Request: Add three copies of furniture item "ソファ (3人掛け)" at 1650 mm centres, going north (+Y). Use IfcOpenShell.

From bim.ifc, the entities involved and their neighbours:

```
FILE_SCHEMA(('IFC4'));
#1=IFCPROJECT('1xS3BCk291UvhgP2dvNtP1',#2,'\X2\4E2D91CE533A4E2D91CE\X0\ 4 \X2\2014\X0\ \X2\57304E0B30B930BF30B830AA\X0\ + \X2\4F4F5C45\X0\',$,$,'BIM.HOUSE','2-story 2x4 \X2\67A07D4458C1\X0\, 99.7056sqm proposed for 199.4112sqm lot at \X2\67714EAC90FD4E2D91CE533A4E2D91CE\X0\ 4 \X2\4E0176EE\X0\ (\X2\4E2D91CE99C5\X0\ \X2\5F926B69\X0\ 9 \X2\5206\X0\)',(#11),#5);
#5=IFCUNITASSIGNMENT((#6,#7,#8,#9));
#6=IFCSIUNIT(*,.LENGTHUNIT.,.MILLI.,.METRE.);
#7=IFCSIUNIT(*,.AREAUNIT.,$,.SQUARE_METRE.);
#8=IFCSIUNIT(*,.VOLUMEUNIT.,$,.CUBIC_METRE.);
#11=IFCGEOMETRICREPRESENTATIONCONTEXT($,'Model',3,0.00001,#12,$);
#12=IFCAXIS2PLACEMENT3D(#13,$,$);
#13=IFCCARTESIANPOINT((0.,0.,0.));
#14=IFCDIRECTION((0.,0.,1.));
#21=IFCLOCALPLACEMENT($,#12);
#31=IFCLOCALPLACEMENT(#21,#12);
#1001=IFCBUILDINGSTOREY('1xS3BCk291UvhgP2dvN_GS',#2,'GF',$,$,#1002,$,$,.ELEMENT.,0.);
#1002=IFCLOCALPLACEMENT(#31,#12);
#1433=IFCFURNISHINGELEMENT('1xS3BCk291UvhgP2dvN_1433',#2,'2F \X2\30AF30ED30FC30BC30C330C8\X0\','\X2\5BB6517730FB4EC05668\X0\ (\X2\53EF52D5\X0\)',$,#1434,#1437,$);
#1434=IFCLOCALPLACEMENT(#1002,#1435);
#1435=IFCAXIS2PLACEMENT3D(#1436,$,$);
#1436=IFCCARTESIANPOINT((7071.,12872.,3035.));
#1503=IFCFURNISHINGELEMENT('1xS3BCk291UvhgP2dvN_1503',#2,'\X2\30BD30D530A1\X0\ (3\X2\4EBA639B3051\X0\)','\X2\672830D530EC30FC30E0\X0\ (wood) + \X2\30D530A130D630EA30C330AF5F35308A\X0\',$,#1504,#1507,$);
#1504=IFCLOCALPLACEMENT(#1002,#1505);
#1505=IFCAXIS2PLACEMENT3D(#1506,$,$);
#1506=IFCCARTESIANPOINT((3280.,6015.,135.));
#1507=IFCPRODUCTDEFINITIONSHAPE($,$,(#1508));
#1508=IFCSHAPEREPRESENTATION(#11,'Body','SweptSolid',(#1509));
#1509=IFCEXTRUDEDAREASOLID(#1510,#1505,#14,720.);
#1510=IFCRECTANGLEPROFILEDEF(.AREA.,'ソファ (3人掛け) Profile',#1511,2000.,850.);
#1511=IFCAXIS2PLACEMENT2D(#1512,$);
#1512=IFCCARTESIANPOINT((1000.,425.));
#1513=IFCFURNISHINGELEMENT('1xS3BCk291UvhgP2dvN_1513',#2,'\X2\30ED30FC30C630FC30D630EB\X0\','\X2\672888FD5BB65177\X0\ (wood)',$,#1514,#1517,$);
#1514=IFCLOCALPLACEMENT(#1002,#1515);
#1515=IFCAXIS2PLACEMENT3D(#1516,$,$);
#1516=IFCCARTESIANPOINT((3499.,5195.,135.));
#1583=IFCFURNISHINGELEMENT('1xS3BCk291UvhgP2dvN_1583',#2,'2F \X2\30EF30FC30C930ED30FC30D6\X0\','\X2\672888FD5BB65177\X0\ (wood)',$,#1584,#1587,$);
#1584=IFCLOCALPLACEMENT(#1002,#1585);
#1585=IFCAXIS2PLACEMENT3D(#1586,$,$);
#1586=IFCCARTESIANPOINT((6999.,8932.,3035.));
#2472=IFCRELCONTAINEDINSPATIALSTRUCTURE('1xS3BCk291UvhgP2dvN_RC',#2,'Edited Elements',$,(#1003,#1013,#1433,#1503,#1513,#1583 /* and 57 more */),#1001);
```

```python
import numpy as np
import ifcopenshell
import ifcopenshell.api.geometry
import ifcopenshell.api.root
import ifcopenshell.util.element
import ifcopenshell.util.placement

model = ifcopenshell.open("bim.ifc")


def reuse_history(source, copy):
    """copy_class also copies each property set's owner history, people and application; keep the originals."""
    for rel in copy.IsDefinedBy:
        if rel.is_a("IfcRelDefinesByProperties") and (history := rel.RelatingPropertyDefinition.OwnerHistory):
            rel.RelatingPropertyDefinition.OwnerHistory = source.OwnerHistory
            ifcopenshell.util.element.remove_deep2(model, history)


source = model.by_guid("1xS3BCk291UvhgP2dvN_1503")
base = ifcopenshell.util.placement.get_local_placement(source.ObjectPlacement)
step = np.array([0.0, 1.0, 0.0]) * 1650.0

for i in range(1, 4):
    copy = ifcopenshell.api.root.copy_class(model, product=source)
    copy.Representation = ifcopenshell.util.element.copy_deep(
        model, source.Representation, exclude=["IfcGeometricRepresentationContext", "IfcRepresentationMap"]
    )
    reuse_history(source, copy)
    matrix = base.copy()
    matrix[:3, 3] += i * step
    print("added at", matrix[:3, 3].round(3) + 0.0)
    ifcopenshell.api.geometry.edit_object_placement(model, product=copy, matrix=matrix, is_si=False)

model.write("bim_edited.ifc")
```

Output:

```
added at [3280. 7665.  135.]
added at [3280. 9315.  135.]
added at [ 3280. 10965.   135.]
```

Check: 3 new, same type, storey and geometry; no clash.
